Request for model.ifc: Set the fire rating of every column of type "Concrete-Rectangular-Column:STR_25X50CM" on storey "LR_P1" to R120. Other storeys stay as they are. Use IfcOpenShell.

First a look at what the model holds.

```python
import ifcopenshell
import ifcopenshell.util.element

model = ifcopenshell.open("model.ifc")
print(model.schema)
storey = next(s for s in model.by_type("IfcBuildingStorey") if s.Name == "LR_P1")
columns = [e for e in ifcopenshell.util.element.get_decomposition(storey) if e.is_a("IfcColumn")]
seen = {}
for e in columns:
    element_type = ifcopenshell.util.element.get_type(e)
    key = (element_type.Name if element_type != e and element_type else None, ifcopenshell.util.element.get_pset(e, "Pset_ColumnCommon", "FireRating"))
    seen[key] = seen.get(key, 0) + 1
for (name, value), count in sorted(seen.items(), key=str):
    print(count, "x", name, "|", value)
```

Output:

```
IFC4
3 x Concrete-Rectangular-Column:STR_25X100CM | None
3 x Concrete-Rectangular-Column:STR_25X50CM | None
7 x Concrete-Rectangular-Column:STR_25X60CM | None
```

```python
import ifcopenshell
import ifcopenshell.api.pset
import ifcopenshell.util.element

model = ifcopenshell.open("model.ifc")

storey = next(s for s in model.by_type("IfcBuildingStorey") if s.Name == "LR_P1")
columns = [e for e in ifcopenshell.util.element.get_decomposition(storey) if e.is_a("IfcColumn")]

count = 0
for e in columns:
    element_type = ifcopenshell.util.element.get_type(e)
    if element_type in (None, e) or element_type.Name != "Concrete-Rectangular-Column:STR_25X50CM":
        continue
    # add_pset returns the element's existing set when there is one.
    pset = ifcopenshell.api.pset.add_pset(model, product=e, name="Pset_ColumnCommon")
    ifcopenshell.api.pset.edit_pset(model, pset=pset, properties={"FireRating": "R120"})
    count += 1

print(count, "columns updated")

model.write("model_edited.ifc")
```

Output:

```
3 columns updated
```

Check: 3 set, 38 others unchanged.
